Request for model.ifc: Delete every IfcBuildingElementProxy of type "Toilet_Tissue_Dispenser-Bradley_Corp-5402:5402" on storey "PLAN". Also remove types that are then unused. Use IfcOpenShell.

First a look at what the model holds.

```python
import ifcopenshell
import ifcopenshell.util.element

model = ifcopenshell.open("model.ifc")
print(model.schema)
storey = next(s for s in model.by_type("IfcBuildingStorey") if s.Name == "PLAN")
proxies = [e for e in ifcopenshell.util.element.get_decomposition(storey) if e.is_a("IfcBuildingElementProxy")]
seen = {}
for e in proxies:
    element_type = ifcopenshell.util.element.get_type(e)
    name = element_type.Name if element_type not in (None, e) else None
    seen[name] = seen.get(name, 0) + 1
for name, count in sorted(seen.items(), key=str):
    print(count, "x", name)
```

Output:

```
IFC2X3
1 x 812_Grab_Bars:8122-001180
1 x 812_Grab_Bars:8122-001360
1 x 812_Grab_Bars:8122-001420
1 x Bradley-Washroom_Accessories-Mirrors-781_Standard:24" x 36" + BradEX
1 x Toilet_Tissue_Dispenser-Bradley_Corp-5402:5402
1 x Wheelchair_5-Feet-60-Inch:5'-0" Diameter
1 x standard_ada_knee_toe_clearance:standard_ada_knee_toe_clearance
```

```python
import ifcopenshell
import ifcopenshell.api.root
import ifcopenshell.util.element

model = ifcopenshell.open("model.ifc")

storey = next(s for s in model.by_type("IfcBuildingStorey") if s.Name == "PLAN")
proxies = [e for e in ifcopenshell.util.element.get_decomposition(storey) if e.is_a("IfcBuildingElementProxy")]
targets = [e for e in proxies if (t := ifcopenshell.util.element.get_type(e)) not in (None, e) and t.Name == "Toilet_Tissue_Dispenser-Bradley_Corp-5402:5402"]
types = {ifcopenshell.util.element.get_type(e) for e in targets} - {None, *targets}

for e in targets:
    ifcopenshell.api.root.remove_product(model, product=e)
print(len(targets), "removed")

unused = [t for t in types if not ifcopenshell.util.element.get_types(t)]
for t in unused:
    ifcopenshell.api.root.remove_product(model, product=t)
print(len(unused), "unused types removed")

model.write("model-out.ifc")
```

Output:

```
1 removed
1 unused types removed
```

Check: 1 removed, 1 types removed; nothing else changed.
